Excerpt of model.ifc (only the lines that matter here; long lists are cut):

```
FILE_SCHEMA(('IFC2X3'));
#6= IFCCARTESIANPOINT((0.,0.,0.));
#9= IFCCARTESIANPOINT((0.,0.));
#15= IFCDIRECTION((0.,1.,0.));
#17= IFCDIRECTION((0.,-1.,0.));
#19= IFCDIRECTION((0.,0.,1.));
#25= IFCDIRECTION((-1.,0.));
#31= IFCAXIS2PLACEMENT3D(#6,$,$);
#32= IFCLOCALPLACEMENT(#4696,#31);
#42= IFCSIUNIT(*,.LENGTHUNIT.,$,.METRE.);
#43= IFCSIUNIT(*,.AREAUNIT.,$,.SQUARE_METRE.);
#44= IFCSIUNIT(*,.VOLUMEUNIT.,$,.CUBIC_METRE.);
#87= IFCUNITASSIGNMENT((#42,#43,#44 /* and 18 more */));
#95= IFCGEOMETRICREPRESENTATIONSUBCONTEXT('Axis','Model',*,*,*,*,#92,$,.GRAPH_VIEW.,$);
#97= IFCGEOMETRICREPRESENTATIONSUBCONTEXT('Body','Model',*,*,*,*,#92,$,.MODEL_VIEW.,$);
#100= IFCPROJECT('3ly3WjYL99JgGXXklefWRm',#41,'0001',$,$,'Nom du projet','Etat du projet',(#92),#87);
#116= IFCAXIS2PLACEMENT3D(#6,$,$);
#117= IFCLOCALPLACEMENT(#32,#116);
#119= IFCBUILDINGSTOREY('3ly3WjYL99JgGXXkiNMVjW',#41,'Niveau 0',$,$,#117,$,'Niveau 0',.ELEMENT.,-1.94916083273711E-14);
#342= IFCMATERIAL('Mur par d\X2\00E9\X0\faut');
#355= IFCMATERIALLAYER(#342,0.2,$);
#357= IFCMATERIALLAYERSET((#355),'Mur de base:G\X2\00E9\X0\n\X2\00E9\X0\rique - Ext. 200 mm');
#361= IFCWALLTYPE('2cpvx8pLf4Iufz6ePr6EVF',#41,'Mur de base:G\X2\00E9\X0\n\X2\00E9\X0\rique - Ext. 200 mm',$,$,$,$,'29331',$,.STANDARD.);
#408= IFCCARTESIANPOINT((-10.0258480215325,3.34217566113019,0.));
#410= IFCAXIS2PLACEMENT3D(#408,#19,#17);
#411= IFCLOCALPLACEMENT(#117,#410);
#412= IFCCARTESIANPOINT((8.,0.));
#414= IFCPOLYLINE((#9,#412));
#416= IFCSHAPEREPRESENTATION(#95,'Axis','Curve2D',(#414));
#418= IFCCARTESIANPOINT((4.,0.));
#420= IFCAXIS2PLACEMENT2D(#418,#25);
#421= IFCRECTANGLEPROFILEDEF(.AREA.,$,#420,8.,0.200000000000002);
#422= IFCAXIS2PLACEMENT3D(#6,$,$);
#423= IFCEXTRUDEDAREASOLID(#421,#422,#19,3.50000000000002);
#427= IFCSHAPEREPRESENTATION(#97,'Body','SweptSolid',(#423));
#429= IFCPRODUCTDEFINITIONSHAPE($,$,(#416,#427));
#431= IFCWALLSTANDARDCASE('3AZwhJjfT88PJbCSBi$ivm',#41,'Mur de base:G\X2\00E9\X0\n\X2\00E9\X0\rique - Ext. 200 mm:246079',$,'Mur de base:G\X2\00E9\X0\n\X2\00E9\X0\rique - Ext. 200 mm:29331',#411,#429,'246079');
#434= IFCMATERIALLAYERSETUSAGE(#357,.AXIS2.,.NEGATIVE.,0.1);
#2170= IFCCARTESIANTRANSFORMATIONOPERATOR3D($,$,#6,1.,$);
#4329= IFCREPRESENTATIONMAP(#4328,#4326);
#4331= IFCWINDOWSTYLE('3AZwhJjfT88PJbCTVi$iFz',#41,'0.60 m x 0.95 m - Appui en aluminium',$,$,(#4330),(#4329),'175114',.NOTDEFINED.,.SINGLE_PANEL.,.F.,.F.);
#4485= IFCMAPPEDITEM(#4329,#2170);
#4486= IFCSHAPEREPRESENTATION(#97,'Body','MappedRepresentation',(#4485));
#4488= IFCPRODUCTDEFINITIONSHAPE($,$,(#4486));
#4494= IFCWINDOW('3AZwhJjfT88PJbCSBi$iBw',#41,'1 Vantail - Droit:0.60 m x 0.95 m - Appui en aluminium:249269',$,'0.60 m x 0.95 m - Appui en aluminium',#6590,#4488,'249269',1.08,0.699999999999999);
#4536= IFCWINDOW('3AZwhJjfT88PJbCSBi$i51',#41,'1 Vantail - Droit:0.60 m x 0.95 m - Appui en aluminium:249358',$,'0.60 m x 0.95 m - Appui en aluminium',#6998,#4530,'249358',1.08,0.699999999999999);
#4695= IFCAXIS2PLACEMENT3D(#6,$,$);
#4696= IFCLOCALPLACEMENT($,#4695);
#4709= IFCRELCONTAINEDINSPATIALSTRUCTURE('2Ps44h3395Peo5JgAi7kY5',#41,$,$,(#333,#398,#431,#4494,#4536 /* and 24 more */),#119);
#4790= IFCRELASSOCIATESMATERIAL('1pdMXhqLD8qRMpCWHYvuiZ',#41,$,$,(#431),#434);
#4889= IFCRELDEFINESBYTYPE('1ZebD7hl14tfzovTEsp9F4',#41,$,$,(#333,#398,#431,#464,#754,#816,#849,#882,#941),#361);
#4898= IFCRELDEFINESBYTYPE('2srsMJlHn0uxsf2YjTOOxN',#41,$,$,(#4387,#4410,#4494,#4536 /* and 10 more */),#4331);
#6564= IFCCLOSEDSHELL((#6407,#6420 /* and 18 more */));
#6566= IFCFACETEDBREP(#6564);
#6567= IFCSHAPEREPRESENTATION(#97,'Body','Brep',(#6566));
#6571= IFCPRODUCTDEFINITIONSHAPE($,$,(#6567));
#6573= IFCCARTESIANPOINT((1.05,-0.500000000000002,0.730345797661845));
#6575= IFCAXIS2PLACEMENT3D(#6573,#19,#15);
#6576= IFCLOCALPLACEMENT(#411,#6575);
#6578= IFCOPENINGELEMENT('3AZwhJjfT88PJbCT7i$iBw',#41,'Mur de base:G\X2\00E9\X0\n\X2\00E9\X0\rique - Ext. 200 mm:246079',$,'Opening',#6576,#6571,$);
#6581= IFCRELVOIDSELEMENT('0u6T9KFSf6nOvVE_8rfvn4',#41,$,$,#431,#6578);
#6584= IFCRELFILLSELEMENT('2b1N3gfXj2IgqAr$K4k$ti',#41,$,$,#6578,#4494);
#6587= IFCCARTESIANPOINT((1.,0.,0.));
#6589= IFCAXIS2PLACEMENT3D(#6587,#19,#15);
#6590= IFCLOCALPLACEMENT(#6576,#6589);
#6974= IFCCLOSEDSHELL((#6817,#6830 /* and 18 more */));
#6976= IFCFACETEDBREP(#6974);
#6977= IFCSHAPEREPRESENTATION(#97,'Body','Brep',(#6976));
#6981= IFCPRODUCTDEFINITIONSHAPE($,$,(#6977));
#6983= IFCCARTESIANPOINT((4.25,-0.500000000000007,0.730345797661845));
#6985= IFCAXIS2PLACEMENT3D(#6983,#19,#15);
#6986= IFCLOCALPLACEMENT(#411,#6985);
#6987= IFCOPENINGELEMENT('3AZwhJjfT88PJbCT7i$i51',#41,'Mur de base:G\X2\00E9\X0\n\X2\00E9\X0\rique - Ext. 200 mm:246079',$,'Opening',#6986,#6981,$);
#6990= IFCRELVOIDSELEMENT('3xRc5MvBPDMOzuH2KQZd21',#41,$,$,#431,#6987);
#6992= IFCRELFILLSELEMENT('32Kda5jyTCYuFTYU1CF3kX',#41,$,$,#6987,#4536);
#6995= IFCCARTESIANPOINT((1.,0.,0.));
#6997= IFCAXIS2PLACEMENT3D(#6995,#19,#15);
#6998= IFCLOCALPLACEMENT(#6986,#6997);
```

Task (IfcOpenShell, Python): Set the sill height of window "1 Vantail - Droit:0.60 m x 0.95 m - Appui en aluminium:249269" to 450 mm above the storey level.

```python
import numpy as np
import ifcopenshell
import ifcopenshell.api.geometry
import ifcopenshell.geom
import ifcopenshell.util.element
import ifcopenshell.util.placement
import ifcopenshell.util.shape
import ifcopenshell.util.unit

model = ifcopenshell.open("model.ifc")
unit_scale = ifcopenshell.util.unit.calculate_unit_scale(model)

window = model.by_guid("3AZwhJjfT88PJbCSBi$iBw")
opening = window.FillsVoids[0].RelatingOpeningElement
storey = ifcopenshell.util.element.get_container(window, ifc_class="IfcBuildingStorey")
level = ifcopenshell.util.placement.get_local_placement(storey.ObjectPlacement)[2, 3]

# The opening's origin need not be at the sill, so measure its lowest point.
shape = ifcopenshell.geom.create_shape(ifcopenshell.geom.settings(), opening)
bottom = ifcopenshell.util.shape.get_shape_bottom_elevation(shape, shape.geometry) / unit_scale
dz = level + 0.45 / unit_scale - bottom

shift = np.array([0.0, 0.0, dz])
# The window is placed relative to its opening, so it follows when the opening moves.
matrix = ifcopenshell.util.placement.get_local_placement(opening.ObjectPlacement)
matrix[:3, 3] += shift
ifcopenshell.api.geometry.edit_object_placement(
    model, product=opening, matrix=matrix, is_si=False, should_transform_children=True
)

print(f"moved by {dz * unit_scale:+.3f} m")

model.write("model_updated.ifc")
```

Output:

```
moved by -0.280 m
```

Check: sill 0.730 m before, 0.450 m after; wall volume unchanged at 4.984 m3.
